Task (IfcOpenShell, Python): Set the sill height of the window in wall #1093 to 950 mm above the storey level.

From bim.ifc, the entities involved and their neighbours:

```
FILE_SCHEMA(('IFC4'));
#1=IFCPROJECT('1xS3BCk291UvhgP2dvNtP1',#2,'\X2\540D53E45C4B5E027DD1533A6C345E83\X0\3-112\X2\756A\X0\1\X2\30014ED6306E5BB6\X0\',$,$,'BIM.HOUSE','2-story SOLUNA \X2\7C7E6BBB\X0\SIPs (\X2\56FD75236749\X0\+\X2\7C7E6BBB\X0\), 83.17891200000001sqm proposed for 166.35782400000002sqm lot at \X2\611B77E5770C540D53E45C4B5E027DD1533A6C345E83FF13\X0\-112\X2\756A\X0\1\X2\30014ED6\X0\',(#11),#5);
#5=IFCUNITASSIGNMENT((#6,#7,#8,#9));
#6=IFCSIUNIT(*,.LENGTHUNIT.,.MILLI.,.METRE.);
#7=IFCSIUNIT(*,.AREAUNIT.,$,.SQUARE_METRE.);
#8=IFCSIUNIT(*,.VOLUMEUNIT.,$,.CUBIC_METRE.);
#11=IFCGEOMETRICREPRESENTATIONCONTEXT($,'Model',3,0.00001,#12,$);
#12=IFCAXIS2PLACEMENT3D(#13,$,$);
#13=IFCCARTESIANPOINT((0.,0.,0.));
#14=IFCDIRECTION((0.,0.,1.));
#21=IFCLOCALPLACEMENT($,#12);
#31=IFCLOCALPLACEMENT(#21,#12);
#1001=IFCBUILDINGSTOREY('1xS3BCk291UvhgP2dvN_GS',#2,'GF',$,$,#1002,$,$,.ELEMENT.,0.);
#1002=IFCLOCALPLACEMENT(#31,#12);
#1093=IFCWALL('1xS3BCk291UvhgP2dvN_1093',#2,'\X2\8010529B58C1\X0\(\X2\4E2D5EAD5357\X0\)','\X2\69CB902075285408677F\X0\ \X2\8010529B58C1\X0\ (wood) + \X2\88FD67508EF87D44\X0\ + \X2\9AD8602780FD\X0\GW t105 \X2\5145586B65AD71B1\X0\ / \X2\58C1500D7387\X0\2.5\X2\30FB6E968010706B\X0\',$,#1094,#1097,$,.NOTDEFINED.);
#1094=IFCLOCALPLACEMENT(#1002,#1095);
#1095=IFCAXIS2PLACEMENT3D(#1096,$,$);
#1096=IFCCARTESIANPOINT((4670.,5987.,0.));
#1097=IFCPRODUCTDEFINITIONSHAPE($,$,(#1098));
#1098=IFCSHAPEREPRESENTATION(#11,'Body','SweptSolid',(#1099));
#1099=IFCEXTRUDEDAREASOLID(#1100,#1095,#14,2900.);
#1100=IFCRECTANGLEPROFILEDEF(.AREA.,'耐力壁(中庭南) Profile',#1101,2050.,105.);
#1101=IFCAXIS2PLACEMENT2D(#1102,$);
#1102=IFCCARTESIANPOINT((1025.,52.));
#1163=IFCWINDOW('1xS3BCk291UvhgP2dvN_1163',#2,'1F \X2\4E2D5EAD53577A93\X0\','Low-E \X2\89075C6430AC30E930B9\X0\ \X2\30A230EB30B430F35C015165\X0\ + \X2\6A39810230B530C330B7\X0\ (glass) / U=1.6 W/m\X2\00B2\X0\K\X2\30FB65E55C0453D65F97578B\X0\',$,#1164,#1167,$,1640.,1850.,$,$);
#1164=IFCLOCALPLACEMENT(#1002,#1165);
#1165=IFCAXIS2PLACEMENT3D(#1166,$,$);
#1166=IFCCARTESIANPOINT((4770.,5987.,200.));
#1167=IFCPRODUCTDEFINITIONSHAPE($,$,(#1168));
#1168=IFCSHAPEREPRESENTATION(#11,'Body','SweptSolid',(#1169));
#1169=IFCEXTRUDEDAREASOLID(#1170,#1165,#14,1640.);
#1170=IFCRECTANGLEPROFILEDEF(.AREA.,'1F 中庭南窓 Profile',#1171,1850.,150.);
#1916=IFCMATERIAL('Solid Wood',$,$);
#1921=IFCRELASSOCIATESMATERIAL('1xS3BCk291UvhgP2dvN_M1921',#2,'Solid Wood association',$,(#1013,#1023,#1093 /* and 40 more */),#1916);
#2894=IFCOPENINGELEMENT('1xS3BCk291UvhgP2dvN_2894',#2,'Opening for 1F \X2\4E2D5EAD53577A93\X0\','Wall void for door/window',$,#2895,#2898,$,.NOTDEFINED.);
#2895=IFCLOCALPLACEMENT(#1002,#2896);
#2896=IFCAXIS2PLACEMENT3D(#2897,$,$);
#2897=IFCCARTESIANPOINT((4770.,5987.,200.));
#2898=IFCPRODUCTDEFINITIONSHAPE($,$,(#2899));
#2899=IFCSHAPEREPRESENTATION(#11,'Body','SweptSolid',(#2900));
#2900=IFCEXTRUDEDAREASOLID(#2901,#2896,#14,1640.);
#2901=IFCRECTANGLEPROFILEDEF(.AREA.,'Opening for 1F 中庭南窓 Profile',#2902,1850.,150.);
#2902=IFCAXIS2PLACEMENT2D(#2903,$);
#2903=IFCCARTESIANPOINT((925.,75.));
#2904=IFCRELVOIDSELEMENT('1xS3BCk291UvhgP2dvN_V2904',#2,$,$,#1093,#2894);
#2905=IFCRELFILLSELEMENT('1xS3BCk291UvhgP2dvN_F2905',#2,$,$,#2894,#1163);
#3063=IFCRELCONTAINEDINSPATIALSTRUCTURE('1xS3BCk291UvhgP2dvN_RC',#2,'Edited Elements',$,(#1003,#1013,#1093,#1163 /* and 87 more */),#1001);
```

```python
import numpy as np
import ifcopenshell
import ifcopenshell.api.geometry
import ifcopenshell.geom
import ifcopenshell.util.element
import ifcopenshell.util.placement
import ifcopenshell.util.shape
import ifcopenshell.util.unit

model = ifcopenshell.open("bim.ifc")
unit_scale = ifcopenshell.util.unit.calculate_unit_scale(model)

window = model.by_guid("1xS3BCk291UvhgP2dvN_1163")
opening = window.FillsVoids[0].RelatingOpeningElement
storey = ifcopenshell.util.element.get_container(window, ifc_class="IfcBuildingStorey")
level = ifcopenshell.util.placement.get_local_placement(storey.ObjectPlacement)[2, 3]

# The opening's origin need not be at the sill, so measure its lowest point.
shape = ifcopenshell.geom.create_shape(ifcopenshell.geom.settings(), opening)
bottom = ifcopenshell.util.shape.get_shape_bottom_elevation(shape, shape.geometry) / unit_scale
dz = level + 950.0 - bottom

shift = np.array([0.0, 0.0, dz])
# The window is not placed relative to its opening, so move both.
for product in (opening, window):
    matrix = ifcopenshell.util.placement.get_local_placement(product.ObjectPlacement)
    matrix[:3, 3] += shift
    ifcopenshell.api.geometry.edit_object_placement(model, product=product, matrix=matrix, is_si=False)

print(f"moved by {dz * unit_scale:+.3f} m")

model.write("bim_rev.ifc")
```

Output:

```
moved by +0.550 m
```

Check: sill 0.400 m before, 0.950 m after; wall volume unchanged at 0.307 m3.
